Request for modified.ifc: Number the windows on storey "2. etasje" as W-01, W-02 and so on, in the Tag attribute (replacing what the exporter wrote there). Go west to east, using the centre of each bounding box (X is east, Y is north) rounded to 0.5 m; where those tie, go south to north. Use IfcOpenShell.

First a look at what the model holds.

```python
import ifcopenshell
import ifcopenshell.util.element
import ifcopenshell.util.placement

model = ifcopenshell.open("modified.ifc")
print(model.schema)
storey = next(s for s in model.by_type("IfcBuildingStorey") if s.Name == "2. etasje")
windows = [e for e in ifcopenshell.util.element.get_decomposition(storey) if e.is_a("IfcWindow")]
for e in sorted(windows, key=lambda e: e.id()):
    origin = ifcopenshell.util.placement.get_local_placement(e.ObjectPlacement)[:3, 3]
    print(e.id(), e.Tag, e.Name, origin.round(2) + 0.0, sep=" | ")
```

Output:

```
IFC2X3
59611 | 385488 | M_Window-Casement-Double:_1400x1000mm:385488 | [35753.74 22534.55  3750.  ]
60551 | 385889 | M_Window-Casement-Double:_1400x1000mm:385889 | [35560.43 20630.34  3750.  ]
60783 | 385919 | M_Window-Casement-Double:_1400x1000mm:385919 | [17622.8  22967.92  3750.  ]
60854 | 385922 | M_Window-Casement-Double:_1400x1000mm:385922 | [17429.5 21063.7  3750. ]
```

```python
import ifcopenshell
import ifcopenshell.geom
import ifcopenshell.util.element
import ifcopenshell.util.shape

model = ifcopenshell.open("modified.ifc")
settings = ifcopenshell.geom.settings()
settings.set("use-world-coords", True)


def centre(element):
    shape = ifcopenshell.geom.create_shape(settings, element)
    return ifcopenshell.util.shape.get_bbox_centroid(shape.geometry)


storey = next(s for s in model.by_type("IfcBuildingStorey") if s.Name == "2. etasje")
windows = [e for e in ifcopenshell.util.element.get_decomposition(storey) if e.is_a("IfcWindow")]

# Insertion points can sit at a corner or the storey origin, so sort by the geometry (in metres).
centres = {e: centre(e) for e in windows}
windows.sort(key=lambda e: (round(centres[e][0] / 0.5), centres[e][1]))

for i, e in enumerate(windows, start=1):
    number = f"W-{i:02d}"
    e.Tag = number
    print(e.id(), number)

model.write("modified-out.ifc")
```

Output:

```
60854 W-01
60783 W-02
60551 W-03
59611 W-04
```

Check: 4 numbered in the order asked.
